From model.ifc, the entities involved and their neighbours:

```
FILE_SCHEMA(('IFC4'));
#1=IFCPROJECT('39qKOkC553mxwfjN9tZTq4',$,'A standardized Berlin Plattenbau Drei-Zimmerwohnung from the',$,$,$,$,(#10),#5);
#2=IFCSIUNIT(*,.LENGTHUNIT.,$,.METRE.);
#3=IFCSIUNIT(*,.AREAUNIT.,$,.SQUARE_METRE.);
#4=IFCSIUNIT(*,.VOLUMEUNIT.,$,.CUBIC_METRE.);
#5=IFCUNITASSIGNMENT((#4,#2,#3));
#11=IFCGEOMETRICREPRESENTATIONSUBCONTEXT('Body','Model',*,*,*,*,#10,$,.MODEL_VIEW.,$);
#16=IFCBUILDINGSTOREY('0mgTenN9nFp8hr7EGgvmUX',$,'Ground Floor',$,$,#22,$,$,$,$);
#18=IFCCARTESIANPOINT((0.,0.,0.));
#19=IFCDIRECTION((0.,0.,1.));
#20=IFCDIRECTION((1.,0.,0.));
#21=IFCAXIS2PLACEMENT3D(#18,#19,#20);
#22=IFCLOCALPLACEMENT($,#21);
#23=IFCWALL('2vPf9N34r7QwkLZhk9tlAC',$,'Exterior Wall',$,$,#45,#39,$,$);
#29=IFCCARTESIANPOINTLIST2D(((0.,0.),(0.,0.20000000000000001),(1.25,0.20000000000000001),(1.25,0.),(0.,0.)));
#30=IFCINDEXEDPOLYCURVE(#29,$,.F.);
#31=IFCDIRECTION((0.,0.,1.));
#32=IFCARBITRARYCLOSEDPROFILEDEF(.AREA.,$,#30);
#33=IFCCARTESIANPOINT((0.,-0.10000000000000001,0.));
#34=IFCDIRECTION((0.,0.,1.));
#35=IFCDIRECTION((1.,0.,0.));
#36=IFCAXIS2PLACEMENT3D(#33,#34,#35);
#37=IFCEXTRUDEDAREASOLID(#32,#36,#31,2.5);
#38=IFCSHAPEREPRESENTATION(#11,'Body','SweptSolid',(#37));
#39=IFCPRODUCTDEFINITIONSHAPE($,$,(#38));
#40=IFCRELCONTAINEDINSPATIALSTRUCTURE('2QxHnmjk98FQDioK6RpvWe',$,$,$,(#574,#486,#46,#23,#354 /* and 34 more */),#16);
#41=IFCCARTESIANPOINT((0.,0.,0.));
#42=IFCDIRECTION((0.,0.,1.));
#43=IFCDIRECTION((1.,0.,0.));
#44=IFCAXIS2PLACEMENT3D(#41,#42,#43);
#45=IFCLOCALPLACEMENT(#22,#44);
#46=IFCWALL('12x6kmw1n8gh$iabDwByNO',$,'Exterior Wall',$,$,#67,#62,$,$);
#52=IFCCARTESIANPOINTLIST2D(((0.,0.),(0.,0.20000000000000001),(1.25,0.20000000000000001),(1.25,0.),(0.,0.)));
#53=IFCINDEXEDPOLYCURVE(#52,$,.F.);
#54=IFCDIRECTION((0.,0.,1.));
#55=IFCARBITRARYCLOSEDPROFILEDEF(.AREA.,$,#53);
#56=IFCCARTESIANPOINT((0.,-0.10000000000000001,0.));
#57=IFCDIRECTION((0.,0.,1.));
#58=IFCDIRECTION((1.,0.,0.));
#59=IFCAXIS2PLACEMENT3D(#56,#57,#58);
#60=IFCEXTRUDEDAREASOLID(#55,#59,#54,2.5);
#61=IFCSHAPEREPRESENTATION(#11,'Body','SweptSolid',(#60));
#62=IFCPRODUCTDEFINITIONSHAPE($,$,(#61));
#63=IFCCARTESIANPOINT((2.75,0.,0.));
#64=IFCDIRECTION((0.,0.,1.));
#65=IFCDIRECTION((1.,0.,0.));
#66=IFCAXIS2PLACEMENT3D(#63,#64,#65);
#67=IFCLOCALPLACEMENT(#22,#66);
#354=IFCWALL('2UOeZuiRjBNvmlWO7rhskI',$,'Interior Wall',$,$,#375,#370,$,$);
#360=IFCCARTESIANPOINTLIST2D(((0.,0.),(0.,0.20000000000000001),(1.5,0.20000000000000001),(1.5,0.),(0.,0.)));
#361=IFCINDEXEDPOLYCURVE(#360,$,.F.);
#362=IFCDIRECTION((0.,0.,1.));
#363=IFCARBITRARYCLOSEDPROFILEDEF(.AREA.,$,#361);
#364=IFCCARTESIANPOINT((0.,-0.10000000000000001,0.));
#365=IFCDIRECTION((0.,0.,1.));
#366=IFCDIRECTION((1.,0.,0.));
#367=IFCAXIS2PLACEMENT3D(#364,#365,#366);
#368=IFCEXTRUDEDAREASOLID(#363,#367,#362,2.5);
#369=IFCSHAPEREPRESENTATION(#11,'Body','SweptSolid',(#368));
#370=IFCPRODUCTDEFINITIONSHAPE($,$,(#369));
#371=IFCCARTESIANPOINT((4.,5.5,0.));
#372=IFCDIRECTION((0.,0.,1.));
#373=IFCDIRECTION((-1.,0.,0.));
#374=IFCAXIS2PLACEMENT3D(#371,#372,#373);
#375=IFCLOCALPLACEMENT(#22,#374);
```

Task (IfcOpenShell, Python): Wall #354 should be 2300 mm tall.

```python
import ifcopenshell
import ifcopenshell.geom
import ifcopenshell.util.representation
import ifcopenshell.util.shape

model = ifcopenshell.open("model.ifc")
settings = ifcopenshell.geom.settings()


def volume(element):
    """Net volume in cubic metres, openings subtracted."""
    shape = ifcopenshell.geom.create_shape(settings, element)
    return ifcopenshell.util.shape.get_volume(shape.geometry)


wall = model.by_guid("2UOeZuiRjBNvmlWO7rhskI")
before = volume(wall)

body = ifcopenshell.util.representation.get_representation(wall, "Model", "Body")
solid = body.Items[0]
old_height = solid.Depth
solid.Depth = 2.3
after = volume(wall)

print(f"height {old_height:g} -> {solid.Depth:g}, volume {before:.3f} -> {after:.3f} m3")

model.write("model_updated.ifc")
```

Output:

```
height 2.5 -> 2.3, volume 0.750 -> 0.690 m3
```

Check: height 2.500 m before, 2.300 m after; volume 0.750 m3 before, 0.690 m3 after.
